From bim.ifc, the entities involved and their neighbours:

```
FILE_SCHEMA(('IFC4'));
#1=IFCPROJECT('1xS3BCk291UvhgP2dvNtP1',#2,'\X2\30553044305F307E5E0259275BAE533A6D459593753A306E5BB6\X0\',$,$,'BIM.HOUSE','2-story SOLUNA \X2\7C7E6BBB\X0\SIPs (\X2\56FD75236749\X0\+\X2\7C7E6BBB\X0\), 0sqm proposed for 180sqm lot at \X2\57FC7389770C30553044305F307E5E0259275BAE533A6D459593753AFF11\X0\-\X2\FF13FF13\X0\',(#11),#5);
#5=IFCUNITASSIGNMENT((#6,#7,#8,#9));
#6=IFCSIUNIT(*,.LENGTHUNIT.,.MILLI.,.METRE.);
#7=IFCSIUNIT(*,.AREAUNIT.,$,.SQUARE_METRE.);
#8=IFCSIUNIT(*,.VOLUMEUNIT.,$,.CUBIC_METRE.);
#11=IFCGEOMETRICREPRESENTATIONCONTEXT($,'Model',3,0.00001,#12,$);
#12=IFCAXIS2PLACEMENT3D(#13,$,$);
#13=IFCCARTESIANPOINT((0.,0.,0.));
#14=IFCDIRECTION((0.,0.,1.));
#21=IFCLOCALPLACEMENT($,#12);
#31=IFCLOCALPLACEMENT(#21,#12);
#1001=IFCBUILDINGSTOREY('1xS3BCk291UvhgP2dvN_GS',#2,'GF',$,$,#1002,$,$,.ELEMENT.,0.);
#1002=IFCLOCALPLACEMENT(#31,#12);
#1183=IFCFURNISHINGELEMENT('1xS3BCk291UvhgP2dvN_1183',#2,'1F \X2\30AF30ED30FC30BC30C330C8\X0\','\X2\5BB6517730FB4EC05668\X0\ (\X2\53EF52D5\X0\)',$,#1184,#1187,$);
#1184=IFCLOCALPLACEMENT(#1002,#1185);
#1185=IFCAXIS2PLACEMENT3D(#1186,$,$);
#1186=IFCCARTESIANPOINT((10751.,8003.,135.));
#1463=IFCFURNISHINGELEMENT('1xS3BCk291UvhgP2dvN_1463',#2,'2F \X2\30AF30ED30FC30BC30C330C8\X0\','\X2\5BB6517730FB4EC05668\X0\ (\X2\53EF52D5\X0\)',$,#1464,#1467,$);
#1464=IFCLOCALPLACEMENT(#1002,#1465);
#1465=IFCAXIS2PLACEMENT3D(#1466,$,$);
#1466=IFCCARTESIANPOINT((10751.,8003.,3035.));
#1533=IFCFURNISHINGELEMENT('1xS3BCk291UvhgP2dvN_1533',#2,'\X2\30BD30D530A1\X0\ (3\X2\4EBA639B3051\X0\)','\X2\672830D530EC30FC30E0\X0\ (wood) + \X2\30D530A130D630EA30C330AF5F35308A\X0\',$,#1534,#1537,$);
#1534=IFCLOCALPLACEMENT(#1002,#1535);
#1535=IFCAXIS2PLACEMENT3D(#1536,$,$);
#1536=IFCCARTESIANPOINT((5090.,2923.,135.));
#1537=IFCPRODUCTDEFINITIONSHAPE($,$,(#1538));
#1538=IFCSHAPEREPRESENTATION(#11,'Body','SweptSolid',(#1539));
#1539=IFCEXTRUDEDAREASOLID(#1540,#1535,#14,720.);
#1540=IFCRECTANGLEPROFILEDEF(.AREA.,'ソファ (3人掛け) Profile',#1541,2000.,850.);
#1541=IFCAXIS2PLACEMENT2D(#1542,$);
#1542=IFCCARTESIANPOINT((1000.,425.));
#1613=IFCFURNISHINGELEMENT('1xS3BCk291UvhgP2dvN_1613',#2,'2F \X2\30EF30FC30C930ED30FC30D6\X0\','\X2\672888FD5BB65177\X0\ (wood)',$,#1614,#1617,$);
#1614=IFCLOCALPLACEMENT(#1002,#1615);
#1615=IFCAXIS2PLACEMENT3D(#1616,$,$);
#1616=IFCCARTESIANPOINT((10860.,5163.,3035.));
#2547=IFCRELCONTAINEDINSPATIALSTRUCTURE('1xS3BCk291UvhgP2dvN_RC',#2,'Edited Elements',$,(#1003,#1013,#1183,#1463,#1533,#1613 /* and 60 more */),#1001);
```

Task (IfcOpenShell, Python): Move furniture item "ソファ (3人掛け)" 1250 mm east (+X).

```python
import ifcopenshell
import ifcopenshell.api.geometry
import ifcopenshell.util.placement

model = ifcopenshell.open("bim.ifc")

item = model.by_guid("1xS3BCk291UvhgP2dvN_1533")
matrix = ifcopenshell.util.placement.get_local_placement(item.ObjectPlacement)
matrix[0, 3] += 1250.0
ifcopenshell.api.geometry.edit_object_placement(model, product=item, matrix=matrix, is_si=False)

print(ifcopenshell.util.placement.get_local_placement(item.ObjectPlacement).round(3) + 0.0)

model.write("bim-out.ifc")
```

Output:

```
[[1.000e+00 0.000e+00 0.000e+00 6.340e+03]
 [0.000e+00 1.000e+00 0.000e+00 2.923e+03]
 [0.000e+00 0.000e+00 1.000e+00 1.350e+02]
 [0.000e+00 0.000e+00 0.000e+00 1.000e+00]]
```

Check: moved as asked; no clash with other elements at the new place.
